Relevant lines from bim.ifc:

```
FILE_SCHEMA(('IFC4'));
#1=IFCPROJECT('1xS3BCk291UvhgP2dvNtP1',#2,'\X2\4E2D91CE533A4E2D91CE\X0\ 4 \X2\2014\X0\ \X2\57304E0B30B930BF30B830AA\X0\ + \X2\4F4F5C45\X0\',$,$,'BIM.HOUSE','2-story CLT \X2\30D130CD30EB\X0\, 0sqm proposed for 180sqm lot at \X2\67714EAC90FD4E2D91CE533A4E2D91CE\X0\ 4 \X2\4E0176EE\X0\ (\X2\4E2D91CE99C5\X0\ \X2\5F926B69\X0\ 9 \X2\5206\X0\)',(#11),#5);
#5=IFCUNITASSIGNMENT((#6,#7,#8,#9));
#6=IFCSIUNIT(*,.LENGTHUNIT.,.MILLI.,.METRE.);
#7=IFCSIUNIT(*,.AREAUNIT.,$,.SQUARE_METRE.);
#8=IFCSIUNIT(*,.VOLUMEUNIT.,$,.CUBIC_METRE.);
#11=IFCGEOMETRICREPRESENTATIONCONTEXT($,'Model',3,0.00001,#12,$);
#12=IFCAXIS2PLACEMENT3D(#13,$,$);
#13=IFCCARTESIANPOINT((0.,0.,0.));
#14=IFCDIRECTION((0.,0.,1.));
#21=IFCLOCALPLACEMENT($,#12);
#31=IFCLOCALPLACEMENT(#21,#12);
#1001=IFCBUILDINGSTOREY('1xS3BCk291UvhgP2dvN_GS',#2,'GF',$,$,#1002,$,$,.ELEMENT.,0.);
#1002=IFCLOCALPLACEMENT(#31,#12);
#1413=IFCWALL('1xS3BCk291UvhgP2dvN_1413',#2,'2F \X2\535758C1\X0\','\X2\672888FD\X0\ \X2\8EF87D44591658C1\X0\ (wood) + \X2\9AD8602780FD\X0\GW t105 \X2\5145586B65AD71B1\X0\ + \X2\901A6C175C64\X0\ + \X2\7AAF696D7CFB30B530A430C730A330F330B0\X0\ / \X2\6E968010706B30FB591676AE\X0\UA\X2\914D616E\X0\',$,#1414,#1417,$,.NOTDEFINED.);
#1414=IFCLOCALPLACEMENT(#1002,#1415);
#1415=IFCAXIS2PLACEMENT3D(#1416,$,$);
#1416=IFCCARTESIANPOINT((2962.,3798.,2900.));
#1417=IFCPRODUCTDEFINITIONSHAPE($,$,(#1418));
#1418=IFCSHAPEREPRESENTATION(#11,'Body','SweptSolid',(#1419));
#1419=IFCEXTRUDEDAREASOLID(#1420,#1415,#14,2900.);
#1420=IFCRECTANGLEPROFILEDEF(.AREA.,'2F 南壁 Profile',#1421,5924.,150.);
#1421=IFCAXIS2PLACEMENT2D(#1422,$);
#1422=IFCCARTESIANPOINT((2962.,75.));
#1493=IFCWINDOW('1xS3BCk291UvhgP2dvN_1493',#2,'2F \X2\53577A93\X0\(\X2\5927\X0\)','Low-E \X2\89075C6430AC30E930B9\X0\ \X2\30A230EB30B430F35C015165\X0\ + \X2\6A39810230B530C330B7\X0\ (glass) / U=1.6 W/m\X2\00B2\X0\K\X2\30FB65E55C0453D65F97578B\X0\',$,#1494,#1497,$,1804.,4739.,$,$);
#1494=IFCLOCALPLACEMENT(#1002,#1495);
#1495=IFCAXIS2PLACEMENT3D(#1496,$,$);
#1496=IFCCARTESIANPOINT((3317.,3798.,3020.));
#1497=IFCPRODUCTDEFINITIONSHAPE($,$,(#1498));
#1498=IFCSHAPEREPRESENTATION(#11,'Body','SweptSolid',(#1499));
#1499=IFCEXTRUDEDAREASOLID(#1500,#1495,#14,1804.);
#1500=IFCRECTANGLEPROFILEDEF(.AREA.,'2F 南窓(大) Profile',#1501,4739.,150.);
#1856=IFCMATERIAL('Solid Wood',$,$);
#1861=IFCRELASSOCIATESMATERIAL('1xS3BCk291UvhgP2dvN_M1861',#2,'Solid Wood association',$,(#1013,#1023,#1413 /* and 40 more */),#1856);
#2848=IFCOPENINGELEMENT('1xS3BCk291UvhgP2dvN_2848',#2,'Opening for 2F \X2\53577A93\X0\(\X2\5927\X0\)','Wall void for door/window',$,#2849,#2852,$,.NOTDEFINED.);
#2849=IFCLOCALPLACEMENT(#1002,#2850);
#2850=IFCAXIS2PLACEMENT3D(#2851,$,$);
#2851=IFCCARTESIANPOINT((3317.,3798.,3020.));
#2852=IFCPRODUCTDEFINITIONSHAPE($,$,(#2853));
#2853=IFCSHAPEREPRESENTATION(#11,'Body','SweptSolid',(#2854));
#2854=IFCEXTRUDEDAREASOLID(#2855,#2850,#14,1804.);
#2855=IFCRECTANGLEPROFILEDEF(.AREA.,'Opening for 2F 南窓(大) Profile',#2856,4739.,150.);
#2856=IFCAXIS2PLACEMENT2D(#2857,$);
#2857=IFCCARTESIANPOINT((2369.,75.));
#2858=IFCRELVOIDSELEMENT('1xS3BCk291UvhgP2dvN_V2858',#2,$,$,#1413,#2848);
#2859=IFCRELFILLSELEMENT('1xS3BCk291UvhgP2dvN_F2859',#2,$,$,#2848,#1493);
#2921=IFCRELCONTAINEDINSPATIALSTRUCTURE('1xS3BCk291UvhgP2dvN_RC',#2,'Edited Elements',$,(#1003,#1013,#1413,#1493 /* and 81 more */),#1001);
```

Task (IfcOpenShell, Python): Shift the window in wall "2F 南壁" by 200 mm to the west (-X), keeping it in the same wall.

```python
import ifcopenshell
import ifcopenshell.api.geometry
import ifcopenshell.util.placement
import ifcopenshell.util.unit

model = ifcopenshell.open("bim.ifc")
unit_scale = ifcopenshell.util.unit.calculate_unit_scale(model)

window = model.by_guid("1xS3BCk291UvhgP2dvN_1493")
opening = window.FillsVoids[0].RelatingOpeningElement
wall = opening.VoidsElements[0].RelatingBuildingElement

wall_matrix = ifcopenshell.util.placement.get_local_placement(wall.ObjectPlacement)
shift = wall_matrix[:3, 0] * -0.2 / unit_scale
before = ifcopenshell.util.placement.get_local_placement(window.ObjectPlacement)[:3, 3].copy()

# The window is not placed relative to its opening, so move both.
for product in (opening, window):
    matrix = ifcopenshell.util.placement.get_local_placement(product.ObjectPlacement)
    matrix[:3, 3] += shift
    ifcopenshell.api.geometry.edit_object_placement(model, product=product, matrix=matrix, is_si=False)

after = ifcopenshell.util.placement.get_local_placement(window.ObjectPlacement)[:3, 3]
print("window moved by", (after - before).round(3) + 0.0)

model.write("bim_v2.ifc")
```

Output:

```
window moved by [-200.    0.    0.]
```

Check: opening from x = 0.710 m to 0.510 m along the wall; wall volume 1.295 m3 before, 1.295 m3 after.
